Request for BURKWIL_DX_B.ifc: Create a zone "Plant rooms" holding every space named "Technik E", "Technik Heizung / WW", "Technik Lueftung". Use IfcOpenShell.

First a look at what the model holds.

```python
import ifcopenshell

model = ifcopenshell.open("BURKWIL_DX_B.ifc")
print(model.schema)
seen = {}
for space in model.by_type("IfcSpace"):
    seen[space.LongName] = seen.get(space.LongName, 0) + 1
for name, count in sorted(seen.items(), key=str):
    print(count, "x", name)
print("zones:", [z.Name for z in model.by_type("IfcZone")][:20])
```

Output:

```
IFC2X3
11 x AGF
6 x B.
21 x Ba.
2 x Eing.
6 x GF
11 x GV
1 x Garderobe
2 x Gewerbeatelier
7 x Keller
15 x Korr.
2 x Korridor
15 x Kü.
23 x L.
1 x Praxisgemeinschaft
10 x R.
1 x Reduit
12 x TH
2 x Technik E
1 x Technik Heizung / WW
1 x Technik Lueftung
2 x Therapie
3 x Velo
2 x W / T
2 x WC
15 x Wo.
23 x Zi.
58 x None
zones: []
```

```python
import ifcopenshell
import ifcopenshell.api.group
import ifcopenshell.api.root

model = ifcopenshell.open("BURKWIL_DX_B.ifc")

names = {"Technik E", "Technik Heizung / WW", "Technik Lueftung"}
spaces = [s for s in model.by_type("IfcSpace") if s.LongName in names]

zone = ifcopenshell.api.root.create_entity(model, ifc_class="IfcZone", name="Plant rooms")
ifcopenshell.api.group.assign_group(model, products=spaces, group=zone)
print(len(spaces), "spaces in", zone.Name)

model.write("BURKWIL_DX_B_updated.ifc")
```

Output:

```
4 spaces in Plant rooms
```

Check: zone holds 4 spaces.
